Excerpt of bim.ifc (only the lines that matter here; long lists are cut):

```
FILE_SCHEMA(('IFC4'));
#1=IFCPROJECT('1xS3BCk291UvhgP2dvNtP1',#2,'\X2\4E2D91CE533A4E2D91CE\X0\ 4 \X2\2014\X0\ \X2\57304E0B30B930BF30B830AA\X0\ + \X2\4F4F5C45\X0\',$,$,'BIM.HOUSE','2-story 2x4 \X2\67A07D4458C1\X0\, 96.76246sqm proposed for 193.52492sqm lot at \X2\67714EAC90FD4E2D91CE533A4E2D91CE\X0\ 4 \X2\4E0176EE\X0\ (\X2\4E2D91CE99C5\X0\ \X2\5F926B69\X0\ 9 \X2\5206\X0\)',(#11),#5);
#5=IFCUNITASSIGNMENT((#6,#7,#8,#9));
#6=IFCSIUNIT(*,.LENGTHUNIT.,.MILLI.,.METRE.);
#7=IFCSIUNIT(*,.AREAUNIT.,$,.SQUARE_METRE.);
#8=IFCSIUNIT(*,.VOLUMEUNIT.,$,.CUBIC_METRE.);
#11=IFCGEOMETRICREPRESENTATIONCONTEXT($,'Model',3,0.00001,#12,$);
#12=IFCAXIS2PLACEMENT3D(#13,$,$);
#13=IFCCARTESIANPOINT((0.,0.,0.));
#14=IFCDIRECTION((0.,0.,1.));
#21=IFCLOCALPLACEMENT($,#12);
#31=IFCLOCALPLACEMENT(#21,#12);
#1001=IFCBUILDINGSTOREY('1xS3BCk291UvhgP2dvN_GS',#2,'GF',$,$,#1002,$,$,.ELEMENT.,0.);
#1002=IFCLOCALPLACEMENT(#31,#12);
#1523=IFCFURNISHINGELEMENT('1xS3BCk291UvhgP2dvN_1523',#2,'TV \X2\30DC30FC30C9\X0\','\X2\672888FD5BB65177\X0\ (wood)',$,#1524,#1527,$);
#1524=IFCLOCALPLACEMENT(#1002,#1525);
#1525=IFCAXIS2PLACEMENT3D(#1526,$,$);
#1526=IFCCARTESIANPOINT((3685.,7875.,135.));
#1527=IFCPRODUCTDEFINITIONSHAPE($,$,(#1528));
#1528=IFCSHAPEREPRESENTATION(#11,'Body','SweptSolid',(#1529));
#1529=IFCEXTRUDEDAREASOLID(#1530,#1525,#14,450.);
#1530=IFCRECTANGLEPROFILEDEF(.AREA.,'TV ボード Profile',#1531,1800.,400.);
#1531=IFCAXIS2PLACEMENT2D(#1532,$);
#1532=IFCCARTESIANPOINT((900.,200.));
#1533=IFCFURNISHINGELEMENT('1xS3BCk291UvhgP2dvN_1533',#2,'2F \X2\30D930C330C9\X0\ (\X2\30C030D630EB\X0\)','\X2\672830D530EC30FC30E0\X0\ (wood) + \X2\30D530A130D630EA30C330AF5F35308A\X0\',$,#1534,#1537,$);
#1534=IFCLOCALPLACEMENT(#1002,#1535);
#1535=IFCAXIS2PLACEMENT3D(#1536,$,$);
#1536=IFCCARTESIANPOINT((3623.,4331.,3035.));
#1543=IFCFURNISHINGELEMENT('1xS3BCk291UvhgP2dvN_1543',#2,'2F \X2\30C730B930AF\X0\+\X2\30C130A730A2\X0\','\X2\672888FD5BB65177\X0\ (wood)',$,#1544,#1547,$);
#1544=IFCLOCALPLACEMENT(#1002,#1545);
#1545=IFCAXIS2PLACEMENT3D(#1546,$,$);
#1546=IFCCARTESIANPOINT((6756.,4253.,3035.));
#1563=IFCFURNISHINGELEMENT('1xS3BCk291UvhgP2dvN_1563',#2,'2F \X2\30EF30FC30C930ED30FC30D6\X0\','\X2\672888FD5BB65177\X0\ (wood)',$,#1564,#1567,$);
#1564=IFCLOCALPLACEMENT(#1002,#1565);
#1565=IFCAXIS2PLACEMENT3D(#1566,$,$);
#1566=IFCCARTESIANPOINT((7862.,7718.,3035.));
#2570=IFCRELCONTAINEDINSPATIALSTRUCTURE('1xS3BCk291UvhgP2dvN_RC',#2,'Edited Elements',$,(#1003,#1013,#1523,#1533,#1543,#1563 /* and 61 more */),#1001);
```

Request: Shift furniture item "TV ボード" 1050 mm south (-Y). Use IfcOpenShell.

```python
import ifcopenshell
import ifcopenshell.api.geometry
import ifcopenshell.util.placement

model = ifcopenshell.open("bim.ifc")

item = model.by_id(1523)
matrix = ifcopenshell.util.placement.get_local_placement(item.ObjectPlacement)
matrix[1, 3] -= 1050.0
ifcopenshell.api.geometry.edit_object_placement(model, product=item, matrix=matrix, is_si=False)

print(ifcopenshell.util.placement.get_local_placement(item.ObjectPlacement).round(3) + 0.0)

model.write("bim_v2.ifc")
```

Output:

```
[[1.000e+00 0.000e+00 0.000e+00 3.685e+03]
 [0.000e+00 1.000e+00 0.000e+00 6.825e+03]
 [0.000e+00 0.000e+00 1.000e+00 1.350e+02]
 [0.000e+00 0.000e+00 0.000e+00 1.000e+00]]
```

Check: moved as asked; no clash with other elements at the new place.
